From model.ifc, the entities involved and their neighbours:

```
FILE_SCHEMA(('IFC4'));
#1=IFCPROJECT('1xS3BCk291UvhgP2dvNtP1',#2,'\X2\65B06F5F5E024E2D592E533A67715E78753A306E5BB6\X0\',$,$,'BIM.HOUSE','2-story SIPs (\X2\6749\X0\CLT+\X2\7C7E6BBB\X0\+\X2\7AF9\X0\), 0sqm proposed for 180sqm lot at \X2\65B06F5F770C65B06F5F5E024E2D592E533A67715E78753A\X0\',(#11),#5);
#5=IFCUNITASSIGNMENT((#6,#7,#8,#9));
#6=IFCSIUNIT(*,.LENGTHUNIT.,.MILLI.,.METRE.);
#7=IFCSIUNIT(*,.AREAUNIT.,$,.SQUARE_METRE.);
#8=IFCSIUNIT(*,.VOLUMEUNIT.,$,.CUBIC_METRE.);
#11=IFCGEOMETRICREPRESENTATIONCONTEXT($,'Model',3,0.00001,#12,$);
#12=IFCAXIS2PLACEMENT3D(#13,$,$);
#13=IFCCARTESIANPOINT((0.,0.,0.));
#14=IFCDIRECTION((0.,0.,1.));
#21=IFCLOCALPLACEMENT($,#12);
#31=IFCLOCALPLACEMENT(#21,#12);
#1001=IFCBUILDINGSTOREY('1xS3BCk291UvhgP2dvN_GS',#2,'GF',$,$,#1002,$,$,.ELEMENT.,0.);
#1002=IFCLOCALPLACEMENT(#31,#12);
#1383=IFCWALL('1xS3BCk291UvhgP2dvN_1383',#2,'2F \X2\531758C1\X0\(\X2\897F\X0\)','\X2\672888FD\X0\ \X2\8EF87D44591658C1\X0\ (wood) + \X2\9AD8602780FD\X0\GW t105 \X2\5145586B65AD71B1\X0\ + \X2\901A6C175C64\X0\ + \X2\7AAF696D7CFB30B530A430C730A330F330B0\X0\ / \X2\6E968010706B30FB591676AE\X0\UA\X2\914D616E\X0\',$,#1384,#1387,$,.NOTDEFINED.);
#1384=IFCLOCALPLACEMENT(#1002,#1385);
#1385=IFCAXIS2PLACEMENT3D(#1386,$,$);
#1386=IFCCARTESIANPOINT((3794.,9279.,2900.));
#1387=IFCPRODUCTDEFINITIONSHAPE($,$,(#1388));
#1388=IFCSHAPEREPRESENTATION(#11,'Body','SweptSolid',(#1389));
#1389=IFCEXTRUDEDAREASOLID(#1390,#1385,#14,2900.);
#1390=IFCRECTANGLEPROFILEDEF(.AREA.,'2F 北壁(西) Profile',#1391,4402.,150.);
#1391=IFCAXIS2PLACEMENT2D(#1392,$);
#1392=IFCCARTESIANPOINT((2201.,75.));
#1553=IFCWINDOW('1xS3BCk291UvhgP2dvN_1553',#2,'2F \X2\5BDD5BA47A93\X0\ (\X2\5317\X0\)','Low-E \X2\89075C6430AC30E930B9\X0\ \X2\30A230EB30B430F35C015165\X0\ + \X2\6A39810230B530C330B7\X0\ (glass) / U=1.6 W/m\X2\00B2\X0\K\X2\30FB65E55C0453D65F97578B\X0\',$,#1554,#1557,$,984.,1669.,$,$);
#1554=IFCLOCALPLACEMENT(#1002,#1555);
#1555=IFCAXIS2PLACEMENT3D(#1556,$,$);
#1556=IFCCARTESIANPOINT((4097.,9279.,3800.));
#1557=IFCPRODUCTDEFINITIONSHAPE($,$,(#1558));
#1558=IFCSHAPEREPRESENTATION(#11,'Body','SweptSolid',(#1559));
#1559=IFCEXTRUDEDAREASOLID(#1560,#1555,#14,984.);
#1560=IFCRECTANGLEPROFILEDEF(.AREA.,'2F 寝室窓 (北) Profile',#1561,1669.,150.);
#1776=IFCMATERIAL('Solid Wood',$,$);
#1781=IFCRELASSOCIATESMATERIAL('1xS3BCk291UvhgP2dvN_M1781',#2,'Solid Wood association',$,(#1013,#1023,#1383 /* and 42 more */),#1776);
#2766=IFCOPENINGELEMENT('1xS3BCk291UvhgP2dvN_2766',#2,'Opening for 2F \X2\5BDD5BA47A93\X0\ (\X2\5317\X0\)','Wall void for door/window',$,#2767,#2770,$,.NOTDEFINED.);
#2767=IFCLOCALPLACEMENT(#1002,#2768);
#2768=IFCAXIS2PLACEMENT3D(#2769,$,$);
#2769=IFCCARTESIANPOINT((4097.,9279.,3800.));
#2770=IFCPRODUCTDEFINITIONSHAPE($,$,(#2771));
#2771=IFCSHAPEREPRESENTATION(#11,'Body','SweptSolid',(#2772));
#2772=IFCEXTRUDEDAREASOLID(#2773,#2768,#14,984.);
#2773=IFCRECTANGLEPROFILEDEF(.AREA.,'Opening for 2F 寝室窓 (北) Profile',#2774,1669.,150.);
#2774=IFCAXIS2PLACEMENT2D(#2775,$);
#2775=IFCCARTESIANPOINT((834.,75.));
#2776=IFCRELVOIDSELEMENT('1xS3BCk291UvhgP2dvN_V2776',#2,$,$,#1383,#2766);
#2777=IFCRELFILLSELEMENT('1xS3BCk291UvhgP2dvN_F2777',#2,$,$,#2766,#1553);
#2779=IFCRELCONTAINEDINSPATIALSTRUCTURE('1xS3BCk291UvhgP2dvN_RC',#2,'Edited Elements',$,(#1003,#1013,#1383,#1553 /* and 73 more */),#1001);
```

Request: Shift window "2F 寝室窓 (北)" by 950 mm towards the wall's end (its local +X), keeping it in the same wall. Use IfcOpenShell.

```python
import ifcopenshell
import ifcopenshell.api.geometry
import ifcopenshell.util.placement

model = ifcopenshell.open("model.ifc")

window = model.by_guid("1xS3BCk291UvhgP2dvN_1553")
opening = window.FillsVoids[0].RelatingOpeningElement
wall = opening.VoidsElements[0].RelatingBuildingElement

wall_matrix = ifcopenshell.util.placement.get_local_placement(wall.ObjectPlacement)
shift = wall_matrix[:3, 0] * 950.0
before = ifcopenshell.util.placement.get_local_placement(window.ObjectPlacement)[:3, 3].copy()

# The window is not placed relative to its opening, so move both.
for product in (opening, window):
    matrix = ifcopenshell.util.placement.get_local_placement(product.ObjectPlacement)
    matrix[:3, 3] += shift
    ifcopenshell.api.geometry.edit_object_placement(model, product=product, matrix=matrix, is_si=False)

after = ifcopenshell.util.placement.get_local_placement(window.ObjectPlacement)[:3, 3]
print("window moved by", (after - before).round(3) + 0.0)

model.write("model_rev.ifc")
```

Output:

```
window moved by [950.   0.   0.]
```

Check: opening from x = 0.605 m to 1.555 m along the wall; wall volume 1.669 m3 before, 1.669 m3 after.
